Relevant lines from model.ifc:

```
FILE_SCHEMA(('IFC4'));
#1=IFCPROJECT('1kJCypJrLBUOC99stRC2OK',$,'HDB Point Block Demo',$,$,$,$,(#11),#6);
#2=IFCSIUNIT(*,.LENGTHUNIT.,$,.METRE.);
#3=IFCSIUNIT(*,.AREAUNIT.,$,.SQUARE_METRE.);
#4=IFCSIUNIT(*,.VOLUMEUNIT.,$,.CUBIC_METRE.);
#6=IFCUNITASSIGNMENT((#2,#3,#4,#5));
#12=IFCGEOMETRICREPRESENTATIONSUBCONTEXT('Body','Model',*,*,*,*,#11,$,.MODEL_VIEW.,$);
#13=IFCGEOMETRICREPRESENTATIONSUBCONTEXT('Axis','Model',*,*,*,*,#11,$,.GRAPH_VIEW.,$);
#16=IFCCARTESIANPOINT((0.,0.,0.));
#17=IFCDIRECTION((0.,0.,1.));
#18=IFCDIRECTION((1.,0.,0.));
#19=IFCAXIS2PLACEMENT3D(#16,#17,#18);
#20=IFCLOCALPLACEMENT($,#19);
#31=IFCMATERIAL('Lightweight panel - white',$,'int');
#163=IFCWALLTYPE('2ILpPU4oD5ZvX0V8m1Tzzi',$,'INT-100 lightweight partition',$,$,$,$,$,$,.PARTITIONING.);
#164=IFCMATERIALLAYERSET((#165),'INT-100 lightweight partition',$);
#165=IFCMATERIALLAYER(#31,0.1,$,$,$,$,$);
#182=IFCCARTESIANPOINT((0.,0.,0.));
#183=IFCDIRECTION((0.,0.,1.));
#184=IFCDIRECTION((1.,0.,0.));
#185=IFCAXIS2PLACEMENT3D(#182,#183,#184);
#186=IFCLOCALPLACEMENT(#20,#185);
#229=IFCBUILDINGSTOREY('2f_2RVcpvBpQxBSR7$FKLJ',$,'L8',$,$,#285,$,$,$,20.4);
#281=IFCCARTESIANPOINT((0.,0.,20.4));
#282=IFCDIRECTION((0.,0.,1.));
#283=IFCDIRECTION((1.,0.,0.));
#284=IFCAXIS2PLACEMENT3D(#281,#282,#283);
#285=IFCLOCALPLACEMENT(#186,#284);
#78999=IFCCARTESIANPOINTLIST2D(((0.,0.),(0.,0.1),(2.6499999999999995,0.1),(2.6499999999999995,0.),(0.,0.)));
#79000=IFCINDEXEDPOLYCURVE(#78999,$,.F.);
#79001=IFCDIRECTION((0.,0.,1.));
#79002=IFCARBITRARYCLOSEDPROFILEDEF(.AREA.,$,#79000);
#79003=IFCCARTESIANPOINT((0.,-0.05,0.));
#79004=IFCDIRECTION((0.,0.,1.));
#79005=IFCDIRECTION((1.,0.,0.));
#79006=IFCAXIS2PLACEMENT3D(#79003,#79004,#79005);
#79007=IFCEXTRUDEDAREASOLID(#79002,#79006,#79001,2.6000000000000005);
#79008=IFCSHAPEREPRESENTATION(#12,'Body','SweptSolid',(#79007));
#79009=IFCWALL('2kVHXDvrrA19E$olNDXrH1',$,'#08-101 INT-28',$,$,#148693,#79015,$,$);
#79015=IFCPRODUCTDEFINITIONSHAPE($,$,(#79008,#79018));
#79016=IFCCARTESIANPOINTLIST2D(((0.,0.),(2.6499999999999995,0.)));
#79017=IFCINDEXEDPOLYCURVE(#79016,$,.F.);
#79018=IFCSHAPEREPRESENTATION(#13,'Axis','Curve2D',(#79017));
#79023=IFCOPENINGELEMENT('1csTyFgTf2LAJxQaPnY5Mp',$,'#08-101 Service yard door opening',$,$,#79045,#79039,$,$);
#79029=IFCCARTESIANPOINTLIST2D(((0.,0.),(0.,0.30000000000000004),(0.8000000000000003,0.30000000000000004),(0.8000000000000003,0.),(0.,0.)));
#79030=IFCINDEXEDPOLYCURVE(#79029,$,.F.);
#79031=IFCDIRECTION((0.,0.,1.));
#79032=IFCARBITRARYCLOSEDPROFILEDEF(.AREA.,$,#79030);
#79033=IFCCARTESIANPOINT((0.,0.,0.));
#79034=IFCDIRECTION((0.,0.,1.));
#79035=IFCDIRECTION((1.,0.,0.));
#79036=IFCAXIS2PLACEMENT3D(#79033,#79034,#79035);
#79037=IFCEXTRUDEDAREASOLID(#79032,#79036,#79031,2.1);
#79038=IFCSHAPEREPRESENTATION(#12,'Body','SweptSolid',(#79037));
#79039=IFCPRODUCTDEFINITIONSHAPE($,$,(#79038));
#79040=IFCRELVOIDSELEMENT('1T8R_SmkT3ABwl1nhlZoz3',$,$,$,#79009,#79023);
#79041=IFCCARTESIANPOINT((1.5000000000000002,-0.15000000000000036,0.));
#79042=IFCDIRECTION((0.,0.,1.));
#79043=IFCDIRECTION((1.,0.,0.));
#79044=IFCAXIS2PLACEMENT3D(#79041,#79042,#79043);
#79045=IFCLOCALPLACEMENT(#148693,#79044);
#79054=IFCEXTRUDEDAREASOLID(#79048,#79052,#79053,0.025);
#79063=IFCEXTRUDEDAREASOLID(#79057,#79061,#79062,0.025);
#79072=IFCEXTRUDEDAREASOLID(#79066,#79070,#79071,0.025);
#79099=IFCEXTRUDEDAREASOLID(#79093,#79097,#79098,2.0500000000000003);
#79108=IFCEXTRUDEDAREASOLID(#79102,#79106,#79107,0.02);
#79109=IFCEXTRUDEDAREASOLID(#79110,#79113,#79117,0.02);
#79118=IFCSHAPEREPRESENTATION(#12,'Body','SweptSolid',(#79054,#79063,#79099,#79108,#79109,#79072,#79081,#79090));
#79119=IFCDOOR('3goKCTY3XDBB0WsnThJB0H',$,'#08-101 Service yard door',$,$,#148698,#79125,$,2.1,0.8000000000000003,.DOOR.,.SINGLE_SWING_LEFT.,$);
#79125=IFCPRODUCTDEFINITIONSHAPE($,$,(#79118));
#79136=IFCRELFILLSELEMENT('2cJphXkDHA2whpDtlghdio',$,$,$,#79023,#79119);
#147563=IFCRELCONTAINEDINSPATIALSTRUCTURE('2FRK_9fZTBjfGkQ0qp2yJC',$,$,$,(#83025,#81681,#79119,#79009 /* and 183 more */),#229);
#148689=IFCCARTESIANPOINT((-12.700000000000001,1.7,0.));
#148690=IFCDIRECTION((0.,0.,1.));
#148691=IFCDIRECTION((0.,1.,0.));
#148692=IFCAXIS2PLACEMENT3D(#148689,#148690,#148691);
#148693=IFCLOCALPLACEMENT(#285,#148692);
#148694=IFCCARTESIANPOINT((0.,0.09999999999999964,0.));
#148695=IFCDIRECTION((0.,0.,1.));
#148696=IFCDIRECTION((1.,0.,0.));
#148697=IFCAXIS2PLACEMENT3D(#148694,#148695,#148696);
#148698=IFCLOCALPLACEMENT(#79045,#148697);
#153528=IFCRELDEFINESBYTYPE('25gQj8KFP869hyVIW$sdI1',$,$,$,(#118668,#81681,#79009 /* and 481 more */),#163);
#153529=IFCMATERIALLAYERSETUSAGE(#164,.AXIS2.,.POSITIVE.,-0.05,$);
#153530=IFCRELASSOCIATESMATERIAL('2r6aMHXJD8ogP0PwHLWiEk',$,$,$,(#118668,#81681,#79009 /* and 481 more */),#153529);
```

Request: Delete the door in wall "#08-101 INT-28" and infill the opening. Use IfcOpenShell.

```python
import ifcopenshell
import ifcopenshell.api.feature
import ifcopenshell.api.root
import ifcopenshell.geom
import ifcopenshell.util.shape

model = ifcopenshell.open("model.ifc")
settings = ifcopenshell.geom.settings()


def volume(element):
    """Net volume in cubic metres, openings subtracted."""
    shape = ifcopenshell.geom.create_shape(settings, element)
    return ifcopenshell.util.shape.get_volume(shape.geometry)


door = model.by_guid("3goKCTY3XDBB0WsnThJB0H")
opening = door.FillsVoids[0].RelatingOpeningElement
wall = opening.VoidsElements[0].RelatingBuildingElement
before = volume(wall)

ifcopenshell.api.root.remove_product(model, product=door)
ifcopenshell.api.feature.remove_feature(model, feature=opening)

after = volume(wall)

print(f"wall volume {before:.3f} -> {after:.3f} m3")

model.write("model_edited.ifc")
```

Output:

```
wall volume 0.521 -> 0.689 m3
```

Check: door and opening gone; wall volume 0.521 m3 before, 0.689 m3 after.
